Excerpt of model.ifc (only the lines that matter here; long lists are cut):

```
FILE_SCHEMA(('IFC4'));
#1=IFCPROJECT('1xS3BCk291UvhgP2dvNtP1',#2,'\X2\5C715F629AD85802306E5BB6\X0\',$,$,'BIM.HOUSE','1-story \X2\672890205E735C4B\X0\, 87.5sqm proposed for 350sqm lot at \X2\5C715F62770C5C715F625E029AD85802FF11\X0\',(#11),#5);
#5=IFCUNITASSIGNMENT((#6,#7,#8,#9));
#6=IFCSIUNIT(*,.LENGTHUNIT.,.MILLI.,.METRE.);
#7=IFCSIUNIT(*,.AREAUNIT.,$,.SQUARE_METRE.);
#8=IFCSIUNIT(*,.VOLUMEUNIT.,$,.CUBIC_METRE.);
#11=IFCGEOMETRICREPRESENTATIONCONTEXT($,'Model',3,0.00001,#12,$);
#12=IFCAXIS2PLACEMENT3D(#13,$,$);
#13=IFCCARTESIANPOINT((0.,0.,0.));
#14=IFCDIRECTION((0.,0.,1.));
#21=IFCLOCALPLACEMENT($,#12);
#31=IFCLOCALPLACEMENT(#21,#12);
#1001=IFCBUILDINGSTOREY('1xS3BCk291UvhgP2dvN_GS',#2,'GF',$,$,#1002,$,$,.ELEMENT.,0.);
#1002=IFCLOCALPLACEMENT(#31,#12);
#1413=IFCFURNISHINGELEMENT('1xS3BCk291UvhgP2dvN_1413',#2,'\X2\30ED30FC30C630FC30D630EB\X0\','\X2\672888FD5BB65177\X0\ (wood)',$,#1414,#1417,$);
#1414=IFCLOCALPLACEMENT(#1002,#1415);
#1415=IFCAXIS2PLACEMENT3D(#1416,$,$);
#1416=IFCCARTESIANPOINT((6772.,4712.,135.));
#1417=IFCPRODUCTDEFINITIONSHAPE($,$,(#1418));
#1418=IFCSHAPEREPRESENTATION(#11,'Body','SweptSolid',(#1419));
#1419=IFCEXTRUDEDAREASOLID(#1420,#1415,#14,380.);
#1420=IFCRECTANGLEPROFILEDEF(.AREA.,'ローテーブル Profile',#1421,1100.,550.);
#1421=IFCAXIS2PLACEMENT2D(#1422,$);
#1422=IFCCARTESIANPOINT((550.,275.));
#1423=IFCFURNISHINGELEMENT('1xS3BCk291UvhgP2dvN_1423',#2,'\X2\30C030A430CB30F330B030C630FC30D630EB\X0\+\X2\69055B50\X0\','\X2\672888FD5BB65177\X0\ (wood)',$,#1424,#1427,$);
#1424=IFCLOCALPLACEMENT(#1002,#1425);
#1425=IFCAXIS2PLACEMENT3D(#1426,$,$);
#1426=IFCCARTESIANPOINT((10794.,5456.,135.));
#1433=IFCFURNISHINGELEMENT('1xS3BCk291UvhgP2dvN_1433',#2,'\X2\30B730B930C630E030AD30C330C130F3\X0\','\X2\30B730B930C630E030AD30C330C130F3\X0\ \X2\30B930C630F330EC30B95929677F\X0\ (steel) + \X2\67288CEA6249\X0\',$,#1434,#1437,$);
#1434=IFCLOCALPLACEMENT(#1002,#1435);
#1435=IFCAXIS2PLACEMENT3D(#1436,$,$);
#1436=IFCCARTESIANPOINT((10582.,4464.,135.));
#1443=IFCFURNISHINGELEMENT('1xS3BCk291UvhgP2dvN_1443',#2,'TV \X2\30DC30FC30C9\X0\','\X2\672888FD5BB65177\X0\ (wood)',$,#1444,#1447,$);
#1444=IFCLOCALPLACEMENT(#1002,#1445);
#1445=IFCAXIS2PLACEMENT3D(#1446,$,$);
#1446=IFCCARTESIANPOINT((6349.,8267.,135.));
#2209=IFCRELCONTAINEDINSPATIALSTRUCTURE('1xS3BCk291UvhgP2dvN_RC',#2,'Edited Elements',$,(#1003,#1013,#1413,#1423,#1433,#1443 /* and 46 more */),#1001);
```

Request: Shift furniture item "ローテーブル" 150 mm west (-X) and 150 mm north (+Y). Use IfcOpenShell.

```python
import ifcopenshell
import ifcopenshell.api.geometry
import ifcopenshell.util.placement

model = ifcopenshell.open("model.ifc")

item = model.by_guid("1xS3BCk291UvhgP2dvN_1413")
matrix = ifcopenshell.util.placement.get_local_placement(item.ObjectPlacement)
matrix[0, 3] -= 150.0
matrix[1, 3] += 150.0
ifcopenshell.api.geometry.edit_object_placement(model, product=item, matrix=matrix, is_si=False)

print(ifcopenshell.util.placement.get_local_placement(item.ObjectPlacement).round(3) + 0.0)

model.write("model-out.ifc")
```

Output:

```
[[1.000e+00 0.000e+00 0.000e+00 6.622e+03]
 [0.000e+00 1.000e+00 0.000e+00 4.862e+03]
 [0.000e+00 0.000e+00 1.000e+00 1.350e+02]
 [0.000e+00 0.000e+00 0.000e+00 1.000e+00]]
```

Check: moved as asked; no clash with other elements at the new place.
